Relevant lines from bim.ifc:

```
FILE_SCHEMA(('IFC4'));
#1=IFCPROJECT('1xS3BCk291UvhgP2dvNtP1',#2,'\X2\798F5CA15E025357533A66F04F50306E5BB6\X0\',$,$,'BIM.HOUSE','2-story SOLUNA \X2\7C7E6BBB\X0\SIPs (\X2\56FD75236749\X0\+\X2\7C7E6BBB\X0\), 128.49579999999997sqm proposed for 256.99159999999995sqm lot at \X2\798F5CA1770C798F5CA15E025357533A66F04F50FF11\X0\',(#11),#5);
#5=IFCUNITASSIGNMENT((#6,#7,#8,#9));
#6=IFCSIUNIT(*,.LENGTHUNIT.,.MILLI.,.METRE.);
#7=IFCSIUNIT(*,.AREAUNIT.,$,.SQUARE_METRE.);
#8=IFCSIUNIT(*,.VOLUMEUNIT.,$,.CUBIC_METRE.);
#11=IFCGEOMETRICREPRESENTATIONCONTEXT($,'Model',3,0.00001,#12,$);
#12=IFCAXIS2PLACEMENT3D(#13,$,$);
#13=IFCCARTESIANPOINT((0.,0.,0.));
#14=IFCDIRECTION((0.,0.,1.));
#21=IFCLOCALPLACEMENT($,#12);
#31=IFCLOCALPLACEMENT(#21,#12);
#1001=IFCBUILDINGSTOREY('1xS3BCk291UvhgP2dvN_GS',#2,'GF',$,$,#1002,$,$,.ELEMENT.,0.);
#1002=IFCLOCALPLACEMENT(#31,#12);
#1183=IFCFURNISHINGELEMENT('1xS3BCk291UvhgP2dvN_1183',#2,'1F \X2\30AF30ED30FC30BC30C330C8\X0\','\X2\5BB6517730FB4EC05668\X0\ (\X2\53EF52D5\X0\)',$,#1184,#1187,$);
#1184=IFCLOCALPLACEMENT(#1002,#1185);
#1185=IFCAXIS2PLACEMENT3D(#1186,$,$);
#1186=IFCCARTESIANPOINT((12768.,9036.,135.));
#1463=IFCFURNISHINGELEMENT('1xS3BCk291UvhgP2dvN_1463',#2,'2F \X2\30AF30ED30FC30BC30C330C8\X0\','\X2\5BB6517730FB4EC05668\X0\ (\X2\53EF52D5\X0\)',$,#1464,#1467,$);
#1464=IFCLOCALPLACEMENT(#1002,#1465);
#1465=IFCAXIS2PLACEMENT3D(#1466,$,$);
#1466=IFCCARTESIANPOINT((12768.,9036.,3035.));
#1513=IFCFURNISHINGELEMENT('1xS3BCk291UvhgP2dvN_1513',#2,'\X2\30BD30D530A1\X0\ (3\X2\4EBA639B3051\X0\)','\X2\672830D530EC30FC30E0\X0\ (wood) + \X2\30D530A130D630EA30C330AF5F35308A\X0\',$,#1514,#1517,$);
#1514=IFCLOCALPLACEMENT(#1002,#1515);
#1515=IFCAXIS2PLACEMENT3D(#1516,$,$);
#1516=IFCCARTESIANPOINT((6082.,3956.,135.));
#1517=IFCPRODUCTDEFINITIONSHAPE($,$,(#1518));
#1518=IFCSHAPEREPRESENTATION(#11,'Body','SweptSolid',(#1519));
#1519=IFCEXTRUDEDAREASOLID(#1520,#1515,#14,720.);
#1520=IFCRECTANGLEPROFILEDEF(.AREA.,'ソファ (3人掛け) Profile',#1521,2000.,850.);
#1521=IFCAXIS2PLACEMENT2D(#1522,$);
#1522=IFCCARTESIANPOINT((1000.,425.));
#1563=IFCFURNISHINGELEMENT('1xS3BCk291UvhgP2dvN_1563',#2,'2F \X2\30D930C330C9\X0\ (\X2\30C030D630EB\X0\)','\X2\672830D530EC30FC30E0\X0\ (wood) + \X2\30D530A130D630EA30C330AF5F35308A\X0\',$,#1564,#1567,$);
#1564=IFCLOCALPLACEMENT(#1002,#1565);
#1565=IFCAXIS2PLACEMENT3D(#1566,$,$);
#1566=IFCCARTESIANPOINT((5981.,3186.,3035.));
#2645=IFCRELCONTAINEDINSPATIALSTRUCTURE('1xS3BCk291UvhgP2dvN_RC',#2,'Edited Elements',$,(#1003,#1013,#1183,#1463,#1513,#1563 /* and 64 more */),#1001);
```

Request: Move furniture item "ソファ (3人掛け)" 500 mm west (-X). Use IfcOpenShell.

```python
import ifcopenshell
import ifcopenshell.api.geometry
import ifcopenshell.util.placement

model = ifcopenshell.open("bim.ifc")

item = model.by_id(1513)
matrix = ifcopenshell.util.placement.get_local_placement(item.ObjectPlacement)
matrix[0, 3] -= 500.0
ifcopenshell.api.geometry.edit_object_placement(model, product=item, matrix=matrix, is_si=False)

print(ifcopenshell.util.placement.get_local_placement(item.ObjectPlacement).round(3) + 0.0)

model.write("bim_rev.ifc")
```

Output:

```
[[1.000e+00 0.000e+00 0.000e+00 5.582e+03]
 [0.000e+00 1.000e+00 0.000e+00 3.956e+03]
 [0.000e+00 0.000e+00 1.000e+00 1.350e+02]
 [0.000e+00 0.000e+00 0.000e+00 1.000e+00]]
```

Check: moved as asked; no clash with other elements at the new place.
